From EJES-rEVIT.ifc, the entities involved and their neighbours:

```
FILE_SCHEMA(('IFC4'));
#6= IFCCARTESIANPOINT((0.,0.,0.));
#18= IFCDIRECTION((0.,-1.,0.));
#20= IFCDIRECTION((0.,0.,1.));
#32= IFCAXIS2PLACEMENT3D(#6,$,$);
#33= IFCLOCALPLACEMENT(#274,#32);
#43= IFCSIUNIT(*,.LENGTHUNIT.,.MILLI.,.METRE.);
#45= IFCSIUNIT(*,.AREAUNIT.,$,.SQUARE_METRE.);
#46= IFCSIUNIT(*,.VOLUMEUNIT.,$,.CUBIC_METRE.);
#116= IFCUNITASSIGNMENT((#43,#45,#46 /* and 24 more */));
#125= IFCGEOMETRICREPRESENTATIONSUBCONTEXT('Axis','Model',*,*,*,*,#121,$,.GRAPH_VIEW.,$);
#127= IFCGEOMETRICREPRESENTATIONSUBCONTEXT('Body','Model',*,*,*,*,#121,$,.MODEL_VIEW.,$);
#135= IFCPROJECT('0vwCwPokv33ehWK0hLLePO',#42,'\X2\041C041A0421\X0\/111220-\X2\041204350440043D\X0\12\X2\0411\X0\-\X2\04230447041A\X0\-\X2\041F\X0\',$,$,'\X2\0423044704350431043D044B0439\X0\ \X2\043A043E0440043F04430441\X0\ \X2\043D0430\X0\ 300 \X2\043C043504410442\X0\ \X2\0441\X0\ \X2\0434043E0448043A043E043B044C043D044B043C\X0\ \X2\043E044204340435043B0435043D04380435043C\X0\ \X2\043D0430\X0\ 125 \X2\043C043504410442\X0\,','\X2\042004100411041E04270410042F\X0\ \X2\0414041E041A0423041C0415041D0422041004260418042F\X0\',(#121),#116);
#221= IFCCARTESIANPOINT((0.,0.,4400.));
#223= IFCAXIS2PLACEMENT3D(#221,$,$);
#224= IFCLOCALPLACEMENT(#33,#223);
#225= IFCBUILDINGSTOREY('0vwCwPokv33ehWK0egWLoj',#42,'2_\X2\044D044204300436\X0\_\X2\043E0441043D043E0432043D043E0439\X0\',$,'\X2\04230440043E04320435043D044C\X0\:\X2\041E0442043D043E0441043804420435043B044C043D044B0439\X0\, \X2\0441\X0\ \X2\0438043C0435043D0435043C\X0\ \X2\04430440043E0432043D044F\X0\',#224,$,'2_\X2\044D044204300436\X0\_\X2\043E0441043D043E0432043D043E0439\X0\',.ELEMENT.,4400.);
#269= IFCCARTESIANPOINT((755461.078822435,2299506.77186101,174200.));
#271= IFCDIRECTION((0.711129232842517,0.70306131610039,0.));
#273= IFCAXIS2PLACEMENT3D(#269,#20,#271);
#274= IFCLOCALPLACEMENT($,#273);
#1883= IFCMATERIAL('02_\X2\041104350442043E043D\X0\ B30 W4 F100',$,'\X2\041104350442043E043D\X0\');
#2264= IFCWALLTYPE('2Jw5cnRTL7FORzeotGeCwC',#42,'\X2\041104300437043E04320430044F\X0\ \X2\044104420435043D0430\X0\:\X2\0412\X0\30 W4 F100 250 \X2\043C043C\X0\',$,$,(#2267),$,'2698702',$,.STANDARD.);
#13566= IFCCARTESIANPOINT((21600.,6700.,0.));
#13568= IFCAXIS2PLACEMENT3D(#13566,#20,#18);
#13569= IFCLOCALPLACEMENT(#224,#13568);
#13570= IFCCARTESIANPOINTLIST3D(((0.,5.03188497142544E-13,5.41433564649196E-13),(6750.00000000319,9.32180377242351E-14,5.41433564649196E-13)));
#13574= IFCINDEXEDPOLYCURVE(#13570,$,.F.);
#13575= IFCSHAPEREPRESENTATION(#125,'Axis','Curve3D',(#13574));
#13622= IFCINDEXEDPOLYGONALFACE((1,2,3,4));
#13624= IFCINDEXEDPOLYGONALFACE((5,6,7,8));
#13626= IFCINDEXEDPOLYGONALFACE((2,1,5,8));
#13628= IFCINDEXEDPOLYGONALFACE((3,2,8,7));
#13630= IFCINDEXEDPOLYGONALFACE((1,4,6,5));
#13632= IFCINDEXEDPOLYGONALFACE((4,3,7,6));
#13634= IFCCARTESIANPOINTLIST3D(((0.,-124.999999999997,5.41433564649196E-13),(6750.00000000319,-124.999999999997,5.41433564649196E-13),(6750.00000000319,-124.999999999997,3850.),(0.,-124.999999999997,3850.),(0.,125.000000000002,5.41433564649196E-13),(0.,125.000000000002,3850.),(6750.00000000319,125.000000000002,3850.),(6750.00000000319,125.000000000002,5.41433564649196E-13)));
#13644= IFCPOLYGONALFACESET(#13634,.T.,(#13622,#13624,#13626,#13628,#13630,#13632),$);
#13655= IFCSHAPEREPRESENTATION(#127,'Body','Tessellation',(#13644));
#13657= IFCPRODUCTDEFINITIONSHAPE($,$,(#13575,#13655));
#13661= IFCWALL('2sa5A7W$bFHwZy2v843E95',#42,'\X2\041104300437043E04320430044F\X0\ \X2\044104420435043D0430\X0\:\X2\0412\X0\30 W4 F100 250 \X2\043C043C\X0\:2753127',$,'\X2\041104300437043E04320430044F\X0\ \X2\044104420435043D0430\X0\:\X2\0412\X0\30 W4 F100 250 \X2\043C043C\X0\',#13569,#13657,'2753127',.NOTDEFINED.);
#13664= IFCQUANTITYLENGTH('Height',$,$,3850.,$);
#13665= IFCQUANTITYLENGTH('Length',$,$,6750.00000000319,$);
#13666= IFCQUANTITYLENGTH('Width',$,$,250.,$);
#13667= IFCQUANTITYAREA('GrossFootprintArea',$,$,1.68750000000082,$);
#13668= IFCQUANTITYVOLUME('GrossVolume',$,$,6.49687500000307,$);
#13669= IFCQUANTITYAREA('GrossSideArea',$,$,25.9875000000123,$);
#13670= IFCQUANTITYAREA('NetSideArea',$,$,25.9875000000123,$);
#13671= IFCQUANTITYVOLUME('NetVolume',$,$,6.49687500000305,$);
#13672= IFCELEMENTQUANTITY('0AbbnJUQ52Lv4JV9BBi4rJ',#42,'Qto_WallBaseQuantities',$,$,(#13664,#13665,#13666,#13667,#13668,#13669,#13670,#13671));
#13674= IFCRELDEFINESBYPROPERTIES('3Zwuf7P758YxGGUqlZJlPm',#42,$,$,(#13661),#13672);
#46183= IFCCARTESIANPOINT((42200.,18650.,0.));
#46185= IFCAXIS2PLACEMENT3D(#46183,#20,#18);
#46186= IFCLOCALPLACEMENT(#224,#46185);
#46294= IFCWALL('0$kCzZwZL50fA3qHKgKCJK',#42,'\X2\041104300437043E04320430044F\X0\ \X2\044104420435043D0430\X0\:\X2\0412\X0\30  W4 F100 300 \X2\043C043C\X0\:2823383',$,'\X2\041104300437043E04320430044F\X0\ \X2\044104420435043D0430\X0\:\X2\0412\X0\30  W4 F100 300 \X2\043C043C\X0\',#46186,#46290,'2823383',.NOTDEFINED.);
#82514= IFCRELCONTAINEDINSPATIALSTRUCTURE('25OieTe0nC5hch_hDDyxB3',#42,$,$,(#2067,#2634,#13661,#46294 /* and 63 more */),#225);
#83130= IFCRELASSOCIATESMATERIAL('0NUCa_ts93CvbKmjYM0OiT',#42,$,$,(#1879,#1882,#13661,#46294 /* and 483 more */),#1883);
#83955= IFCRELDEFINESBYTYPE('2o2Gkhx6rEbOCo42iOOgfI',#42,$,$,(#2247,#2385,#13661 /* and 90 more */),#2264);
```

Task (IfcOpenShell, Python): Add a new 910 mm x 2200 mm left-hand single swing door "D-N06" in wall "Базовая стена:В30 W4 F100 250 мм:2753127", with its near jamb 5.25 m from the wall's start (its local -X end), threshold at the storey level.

```python
import numpy as np
import ifcopenshell
import ifcopenshell.api.feature
import ifcopenshell.api.geometry
import ifcopenshell.api.pset
import ifcopenshell.api.root
import ifcopenshell.api.spatial
import ifcopenshell.geom
import ifcopenshell.util.element
import ifcopenshell.util.placement
import ifcopenshell.util.representation
import ifcopenshell.util.shape
import ifcopenshell.util.unit

model = ifcopenshell.open("EJES-rEVIT.ifc")
unit_scale = ifcopenshell.util.unit.calculate_unit_scale(model)
area_scale = ifcopenshell.util.unit.calculate_unit_scale(model, "AREAUNIT")
volume_scale = ifcopenshell.util.unit.calculate_unit_scale(model, "VOLUMEUNIT")
settings = ifcopenshell.geom.settings()


def volume(element):
    """Net volume in cubic metres, openings subtracted."""
    shape = ifcopenshell.geom.create_shape(settings, element)
    return ifcopenshell.util.shape.get_volume(shape.geometry)


wall = model.by_guid("2sa5A7W$bFHwZy2v843E95")
storey = ifcopenshell.util.element.get_container(wall, ifc_class="IfcBuildingStorey")
context = ifcopenshell.util.representation.get_context(model, "Model", "Body", "MODEL_VIEW")
before = volume(wall)

width, height, from_end, sill = 0.91, 2.2, 5.25, 0.0  # metres

# The wall runs along its own X axis, and the end named is its -X end.
wall_shape = ifcopenshell.geom.create_shape(settings, wall)
x, y, z = ifcopenshell.util.shape.get_vertices(wall_shape.geometry).T
start = x.min() + from_end
face, thickness = float(y.min()), float(y.max() - y.min())
wall_matrix = ifcopenshell.util.placement.get_local_placement(wall.ObjectPlacement)
level = ifcopenshell.util.placement.get_local_placement(storey.ObjectPlacement)[2, 3]


def in_wall(x, y):
    """Placement at x, y metres in the wall's axes, at sill height."""
    matrix = wall_matrix.copy()
    matrix[:, 3] = wall_matrix @ np.array([x / unit_scale, y / unit_scale, 0.0, 1.0])
    matrix[2, 3] = level + sill / unit_scale
    return matrix


# Opening: a box that overshoots both wall faces by 50 mm.
opening = ifcopenshell.api.root.create_entity(model, ifc_class="IfcOpeningElement", predefined_type="OPENING")
box = ifcopenshell.api.geometry.add_wall_representation(
    model, context=context, length=width, height=height, thickness=thickness + 0.1
)
ifcopenshell.api.geometry.assign_representation(model, product=opening, representation=box)
ifcopenshell.api.geometry.edit_object_placement(model, product=opening, matrix=in_wall(start, face - 0.05), is_si=False)
ifcopenshell.api.feature.add_feature(model, feature=opening, element=wall)

door = ifcopenshell.api.root.create_entity(model, ifc_class="IfcDoor", name="D-N06", predefined_type="DOOR")
door.OverallWidth, door.OverallHeight = width / unit_scale, height / unit_scale
door.OperationType = "SINGLE_SWING_LEFT"
body = ifcopenshell.api.geometry.add_door_representation(
    model,
    context=context,
    overall_width=door.OverallWidth,
    overall_height=door.OverallHeight,
    operation_type="SINGLE_SWING_LEFT",
    lining_properties={"LiningDepth": thickness / unit_scale, "ThresholdDepth": thickness / unit_scale},
)
ifcopenshell.api.geometry.assign_representation(model, product=door, representation=body)
ifcopenshell.api.spatial.assign_container(model, products=[door], relating_structure=storey)
ifcopenshell.api.feature.add_filling(model, opening=opening, element=door)

# The lining spans the wall, so the door starts at the wall face.
ifcopenshell.api.geometry.edit_object_placement(model, product=door, matrix=in_wall(start, face), is_si=False)

after = volume(wall)

# Update the wall's stored quantities.
qto = model.by_id(ifcopenshell.util.element.get_pset(wall, "Qto_WallBaseQuantities", should_inherit=False)["id"])
ifcopenshell.api.pset.edit_qto(model, qto=qto, properties={
    "NetSideArea": after / thickness / area_scale,
    "NetVolume": after / volume_scale,
})

print(f"wall volume {before:.3f} -> {after:.3f} m3")

model.write("EJES-rEVIT_v2.ifc")
```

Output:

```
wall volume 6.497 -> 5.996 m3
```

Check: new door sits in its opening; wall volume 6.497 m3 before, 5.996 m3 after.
